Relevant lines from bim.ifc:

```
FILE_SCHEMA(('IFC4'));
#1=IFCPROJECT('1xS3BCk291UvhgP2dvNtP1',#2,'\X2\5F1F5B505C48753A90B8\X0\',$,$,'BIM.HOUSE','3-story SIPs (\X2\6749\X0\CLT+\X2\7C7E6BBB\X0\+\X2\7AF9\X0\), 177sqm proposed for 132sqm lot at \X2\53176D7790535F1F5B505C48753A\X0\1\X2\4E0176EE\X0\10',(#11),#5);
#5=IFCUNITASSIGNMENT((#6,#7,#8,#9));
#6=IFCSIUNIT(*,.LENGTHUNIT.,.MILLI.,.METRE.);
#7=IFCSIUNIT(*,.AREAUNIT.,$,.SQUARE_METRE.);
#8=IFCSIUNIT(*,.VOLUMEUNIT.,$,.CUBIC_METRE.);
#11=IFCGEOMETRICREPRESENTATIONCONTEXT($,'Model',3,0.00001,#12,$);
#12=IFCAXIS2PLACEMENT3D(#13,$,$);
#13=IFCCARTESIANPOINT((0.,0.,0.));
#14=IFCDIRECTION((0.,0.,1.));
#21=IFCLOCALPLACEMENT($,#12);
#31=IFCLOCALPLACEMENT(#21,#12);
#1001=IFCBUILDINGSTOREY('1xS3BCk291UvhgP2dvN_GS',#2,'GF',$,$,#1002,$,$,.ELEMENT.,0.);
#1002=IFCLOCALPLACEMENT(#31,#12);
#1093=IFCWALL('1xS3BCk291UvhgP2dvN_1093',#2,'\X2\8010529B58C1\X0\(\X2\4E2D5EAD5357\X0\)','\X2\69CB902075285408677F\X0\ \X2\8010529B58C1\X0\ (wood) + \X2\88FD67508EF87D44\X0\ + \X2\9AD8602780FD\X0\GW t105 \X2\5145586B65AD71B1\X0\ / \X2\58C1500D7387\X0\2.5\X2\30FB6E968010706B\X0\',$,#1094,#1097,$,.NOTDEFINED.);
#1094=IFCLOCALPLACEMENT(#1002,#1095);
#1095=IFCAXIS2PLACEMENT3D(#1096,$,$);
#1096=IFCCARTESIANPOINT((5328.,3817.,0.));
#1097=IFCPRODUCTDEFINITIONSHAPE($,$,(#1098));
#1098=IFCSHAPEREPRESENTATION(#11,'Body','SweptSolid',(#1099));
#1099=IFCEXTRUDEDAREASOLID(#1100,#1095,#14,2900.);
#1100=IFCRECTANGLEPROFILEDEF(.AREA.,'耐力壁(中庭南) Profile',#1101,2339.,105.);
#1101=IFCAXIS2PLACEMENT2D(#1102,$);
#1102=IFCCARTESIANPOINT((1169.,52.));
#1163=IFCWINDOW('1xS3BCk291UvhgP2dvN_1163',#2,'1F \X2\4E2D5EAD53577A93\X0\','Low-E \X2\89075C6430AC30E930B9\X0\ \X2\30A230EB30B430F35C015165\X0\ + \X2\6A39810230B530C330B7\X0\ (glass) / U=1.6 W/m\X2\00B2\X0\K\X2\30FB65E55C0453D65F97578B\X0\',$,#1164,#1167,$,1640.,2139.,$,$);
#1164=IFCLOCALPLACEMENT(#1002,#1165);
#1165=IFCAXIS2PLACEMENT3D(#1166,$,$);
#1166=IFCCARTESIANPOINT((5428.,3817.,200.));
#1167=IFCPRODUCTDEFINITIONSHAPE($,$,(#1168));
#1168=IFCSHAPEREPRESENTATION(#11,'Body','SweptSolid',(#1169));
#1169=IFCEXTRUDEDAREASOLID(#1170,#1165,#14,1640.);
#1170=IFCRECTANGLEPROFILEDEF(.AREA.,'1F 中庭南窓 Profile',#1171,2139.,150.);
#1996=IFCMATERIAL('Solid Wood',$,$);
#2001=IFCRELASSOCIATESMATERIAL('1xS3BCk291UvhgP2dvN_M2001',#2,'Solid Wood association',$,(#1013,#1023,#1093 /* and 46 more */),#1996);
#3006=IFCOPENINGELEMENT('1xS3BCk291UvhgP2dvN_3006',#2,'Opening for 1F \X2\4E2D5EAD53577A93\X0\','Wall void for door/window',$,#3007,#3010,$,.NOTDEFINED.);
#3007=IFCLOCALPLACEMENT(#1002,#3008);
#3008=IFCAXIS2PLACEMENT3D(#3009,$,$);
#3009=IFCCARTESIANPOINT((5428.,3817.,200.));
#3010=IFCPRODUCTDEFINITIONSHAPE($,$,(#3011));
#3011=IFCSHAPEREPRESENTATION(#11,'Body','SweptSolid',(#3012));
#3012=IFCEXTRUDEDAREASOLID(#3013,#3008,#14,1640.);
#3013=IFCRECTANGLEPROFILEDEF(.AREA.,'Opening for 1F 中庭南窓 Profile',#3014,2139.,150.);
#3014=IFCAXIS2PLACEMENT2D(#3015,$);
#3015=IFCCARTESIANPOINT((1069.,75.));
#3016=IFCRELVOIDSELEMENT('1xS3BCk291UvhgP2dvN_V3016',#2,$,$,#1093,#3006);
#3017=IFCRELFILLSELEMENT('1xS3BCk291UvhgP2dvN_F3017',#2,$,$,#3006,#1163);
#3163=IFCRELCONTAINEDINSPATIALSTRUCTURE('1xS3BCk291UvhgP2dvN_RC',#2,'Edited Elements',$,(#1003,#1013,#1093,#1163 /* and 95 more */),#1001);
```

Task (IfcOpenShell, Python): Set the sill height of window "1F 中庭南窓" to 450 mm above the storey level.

```python
import numpy as np
import ifcopenshell
import ifcopenshell.api.geometry
import ifcopenshell.geom
import ifcopenshell.util.element
import ifcopenshell.util.placement
import ifcopenshell.util.shape
import ifcopenshell.util.unit

model = ifcopenshell.open("bim.ifc")
unit_scale = ifcopenshell.util.unit.calculate_unit_scale(model)

window = model.by_guid("1xS3BCk291UvhgP2dvN_1163")
opening = window.FillsVoids[0].RelatingOpeningElement
storey = ifcopenshell.util.element.get_container(window, ifc_class="IfcBuildingStorey")
level = ifcopenshell.util.placement.get_local_placement(storey.ObjectPlacement)[2, 3]

# The opening's origin need not be at the sill, so measure its lowest point.
shape = ifcopenshell.geom.create_shape(ifcopenshell.geom.settings(), opening)
bottom = ifcopenshell.util.shape.get_shape_bottom_elevation(shape, shape.geometry) / unit_scale
dz = level + 0.45 / unit_scale - bottom

shift = np.array([0.0, 0.0, dz])
# The window is not placed relative to its opening, so move both.
for product in (opening, window):
    matrix = ifcopenshell.util.placement.get_local_placement(product.ObjectPlacement)
    matrix[:3, 3] += shift
    ifcopenshell.api.geometry.edit_object_placement(model, product=product, matrix=matrix, is_si=False)

print(f"moved by {dz * unit_scale:+.3f} m")

model.write("bim_edited.ifc")
```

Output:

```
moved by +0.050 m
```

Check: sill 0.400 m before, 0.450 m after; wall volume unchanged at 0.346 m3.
